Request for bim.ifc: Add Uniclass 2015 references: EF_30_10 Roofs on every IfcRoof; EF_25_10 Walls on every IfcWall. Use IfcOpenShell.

First a look at what the model holds.

```python
import ifcopenshell

model = ifcopenshell.open("bim.ifc")
print(model.schema)
print("classifications:", [c.Name for c in model.by_type("IfcClassification")])
for ifc_class in ("IfcDoor", "IfcRoof", "IfcStair", "IfcWall", "IfcWindow"):
    print(ifc_class, len(model.by_type(ifc_class)))
```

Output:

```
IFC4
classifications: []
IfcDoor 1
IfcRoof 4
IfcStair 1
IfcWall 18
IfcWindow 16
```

```python
import ifcopenshell
import ifcopenshell.api.classification

model = ifcopenshell.open("bim.ifc")

system = ifcopenshell.api.classification.add_classification(model, classification="Uniclass 2015")

codes = {
    "IfcRoof": ("EF_30_10", "Roofs"),
    "IfcWall": ("EF_25_10", "Walls"),
}
for ifc_class, (code, name) in codes.items():
    products = model.by_type(ifc_class)
    ifcopenshell.api.classification.add_reference(
        model, products=products, classification=system, identification=code, name=name
    )
    print(code, len(products))

model.write("bim_edited.ifc")
```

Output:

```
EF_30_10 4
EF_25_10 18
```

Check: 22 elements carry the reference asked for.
